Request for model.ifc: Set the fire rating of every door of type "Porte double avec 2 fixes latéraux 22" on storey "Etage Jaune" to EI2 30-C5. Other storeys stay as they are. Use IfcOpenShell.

First a look at what the model holds.

```python
import ifcopenshell
import ifcopenshell.util.element

model = ifcopenshell.open("model.ifc")
print(model.schema)
storey = next(s for s in model.by_type("IfcBuildingStorey") if s.Name == "Etage Jaune")
doors = [e for e in ifcopenshell.util.element.get_decomposition(storey) if e.is_a("IfcDoor")]
seen = {}
for e in doors:
    element_type = ifcopenshell.util.element.get_type(e)
    key = (element_type.Name if element_type != e and element_type else None, ifcopenshell.util.element.get_pset(e, "Pset_DoorCommon", "FireRating"))
    seen[key] = seen.get(key, 0) + 1
for (name, value), count in sorted(seen.items(), key=str):
    print(count, "x", name, "|", value)
```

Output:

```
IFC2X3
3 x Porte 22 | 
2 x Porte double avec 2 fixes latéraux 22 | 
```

```python
import ifcopenshell
import ifcopenshell.api.pset
import ifcopenshell.util.element

model = ifcopenshell.open("model.ifc")

storey = next(s for s in model.by_type("IfcBuildingStorey") if s.Name == "Etage Jaune")
doors = [e for e in ifcopenshell.util.element.get_decomposition(storey) if e.is_a("IfcDoor")]

count = 0
for e in doors:
    element_type = ifcopenshell.util.element.get_type(e)
    if element_type in (None, e) or element_type.Name != "Porte double avec 2 fixes latéraux 22":
        continue
    # add_pset returns the element's existing set when there is one.
    pset = ifcopenshell.api.pset.add_pset(model, product=e, name="Pset_DoorCommon")
    ifcopenshell.api.pset.edit_pset(model, pset=pset, properties={"FireRating": "EI2 30-C5"})
    count += 1

print(count, "doors updated")

model.write("model_updated.ifc")
```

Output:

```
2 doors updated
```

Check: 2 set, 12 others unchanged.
